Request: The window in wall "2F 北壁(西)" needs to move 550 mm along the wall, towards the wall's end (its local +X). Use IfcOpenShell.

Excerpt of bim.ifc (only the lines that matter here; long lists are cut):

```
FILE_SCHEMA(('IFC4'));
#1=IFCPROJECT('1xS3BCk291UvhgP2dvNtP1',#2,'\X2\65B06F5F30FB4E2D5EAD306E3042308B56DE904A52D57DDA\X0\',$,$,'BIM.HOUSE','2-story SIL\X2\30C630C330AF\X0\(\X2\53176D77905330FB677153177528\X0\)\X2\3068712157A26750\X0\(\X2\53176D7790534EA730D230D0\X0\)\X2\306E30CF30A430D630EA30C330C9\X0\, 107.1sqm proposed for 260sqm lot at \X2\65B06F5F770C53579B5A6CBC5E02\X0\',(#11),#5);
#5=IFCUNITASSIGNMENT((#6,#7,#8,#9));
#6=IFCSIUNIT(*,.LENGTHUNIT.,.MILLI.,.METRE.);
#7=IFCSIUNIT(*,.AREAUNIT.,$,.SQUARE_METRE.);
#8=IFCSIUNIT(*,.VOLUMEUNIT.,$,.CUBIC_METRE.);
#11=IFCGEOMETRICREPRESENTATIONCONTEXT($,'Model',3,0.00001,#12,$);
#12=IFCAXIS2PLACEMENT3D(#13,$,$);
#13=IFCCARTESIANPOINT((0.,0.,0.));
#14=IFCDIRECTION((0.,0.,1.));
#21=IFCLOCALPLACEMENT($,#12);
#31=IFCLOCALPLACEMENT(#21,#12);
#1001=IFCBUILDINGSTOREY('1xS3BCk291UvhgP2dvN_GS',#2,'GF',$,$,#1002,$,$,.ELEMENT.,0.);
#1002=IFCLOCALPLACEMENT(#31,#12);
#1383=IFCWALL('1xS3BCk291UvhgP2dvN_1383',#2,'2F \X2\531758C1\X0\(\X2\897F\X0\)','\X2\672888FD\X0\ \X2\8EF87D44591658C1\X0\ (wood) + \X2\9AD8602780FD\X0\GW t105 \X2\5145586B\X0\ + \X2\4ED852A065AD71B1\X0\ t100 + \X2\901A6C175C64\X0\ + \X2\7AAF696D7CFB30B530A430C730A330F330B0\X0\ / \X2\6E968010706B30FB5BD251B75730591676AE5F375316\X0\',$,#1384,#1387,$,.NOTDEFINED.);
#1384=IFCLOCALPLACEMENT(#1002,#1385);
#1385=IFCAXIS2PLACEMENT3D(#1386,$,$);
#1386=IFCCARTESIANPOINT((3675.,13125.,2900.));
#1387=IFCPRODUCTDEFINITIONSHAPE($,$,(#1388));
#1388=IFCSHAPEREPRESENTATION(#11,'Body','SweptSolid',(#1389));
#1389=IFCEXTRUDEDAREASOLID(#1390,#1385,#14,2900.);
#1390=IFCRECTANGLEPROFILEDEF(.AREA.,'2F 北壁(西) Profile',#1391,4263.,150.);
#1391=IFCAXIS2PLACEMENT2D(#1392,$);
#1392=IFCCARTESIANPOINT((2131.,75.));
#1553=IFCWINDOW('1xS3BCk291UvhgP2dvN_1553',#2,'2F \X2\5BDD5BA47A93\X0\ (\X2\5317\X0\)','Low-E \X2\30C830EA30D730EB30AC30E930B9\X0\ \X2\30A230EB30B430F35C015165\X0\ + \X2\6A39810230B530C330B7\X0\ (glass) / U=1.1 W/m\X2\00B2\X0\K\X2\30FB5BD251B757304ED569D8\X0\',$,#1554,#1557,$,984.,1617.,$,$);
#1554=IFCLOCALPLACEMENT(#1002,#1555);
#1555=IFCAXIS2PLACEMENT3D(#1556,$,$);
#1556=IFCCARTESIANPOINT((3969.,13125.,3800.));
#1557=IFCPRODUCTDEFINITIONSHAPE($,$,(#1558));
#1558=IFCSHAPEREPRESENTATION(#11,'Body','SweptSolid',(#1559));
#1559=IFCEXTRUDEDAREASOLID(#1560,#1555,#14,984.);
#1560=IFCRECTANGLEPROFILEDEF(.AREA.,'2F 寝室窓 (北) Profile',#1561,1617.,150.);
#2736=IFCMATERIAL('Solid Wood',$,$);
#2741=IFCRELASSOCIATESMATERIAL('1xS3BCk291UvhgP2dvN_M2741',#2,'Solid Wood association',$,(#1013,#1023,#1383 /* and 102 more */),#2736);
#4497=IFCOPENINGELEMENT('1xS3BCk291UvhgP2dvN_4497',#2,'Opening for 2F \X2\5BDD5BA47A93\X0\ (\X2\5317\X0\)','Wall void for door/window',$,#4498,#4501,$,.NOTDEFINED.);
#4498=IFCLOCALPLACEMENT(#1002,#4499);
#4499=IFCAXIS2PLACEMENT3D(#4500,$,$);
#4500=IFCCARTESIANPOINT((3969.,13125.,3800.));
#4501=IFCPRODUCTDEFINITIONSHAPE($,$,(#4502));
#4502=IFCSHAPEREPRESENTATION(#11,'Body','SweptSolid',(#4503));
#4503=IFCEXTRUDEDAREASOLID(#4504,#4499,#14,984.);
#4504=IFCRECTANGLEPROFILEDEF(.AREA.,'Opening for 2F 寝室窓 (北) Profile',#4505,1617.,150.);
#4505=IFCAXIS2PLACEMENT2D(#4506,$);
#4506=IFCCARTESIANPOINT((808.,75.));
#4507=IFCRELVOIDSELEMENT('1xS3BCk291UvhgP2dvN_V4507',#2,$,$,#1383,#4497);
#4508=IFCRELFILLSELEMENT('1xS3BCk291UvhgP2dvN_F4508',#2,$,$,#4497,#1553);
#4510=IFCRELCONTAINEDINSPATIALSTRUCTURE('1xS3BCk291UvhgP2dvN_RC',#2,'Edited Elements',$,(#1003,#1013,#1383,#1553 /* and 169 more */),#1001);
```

```python
import ifcopenshell
import ifcopenshell.api.geometry
import ifcopenshell.util.placement
import ifcopenshell.util.unit

model = ifcopenshell.open("bim.ifc")
unit_scale = ifcopenshell.util.unit.calculate_unit_scale(model)

window = model.by_guid("1xS3BCk291UvhgP2dvN_1553")
opening = window.FillsVoids[0].RelatingOpeningElement
wall = opening.VoidsElements[0].RelatingBuildingElement

wall_matrix = ifcopenshell.util.placement.get_local_placement(wall.ObjectPlacement)
shift = wall_matrix[:3, 0] * 0.55 / unit_scale
before = ifcopenshell.util.placement.get_local_placement(window.ObjectPlacement)[:3, 3].copy()

# The window is not placed relative to its opening, so move both.
for product in (opening, window):
    matrix = ifcopenshell.util.placement.get_local_placement(product.ObjectPlacement)
    matrix[:3, 3] += shift
    ifcopenshell.api.geometry.edit_object_placement(model, product=product, matrix=matrix, is_si=False)

after = ifcopenshell.util.placement.get_local_placement(window.ObjectPlacement)[:3, 3]
print("window moved by", (after - before).round(3) + 0.0)

model.write("bim_edited.ifc")
```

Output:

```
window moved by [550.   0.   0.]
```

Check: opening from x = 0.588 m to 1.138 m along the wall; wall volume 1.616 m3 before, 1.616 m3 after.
